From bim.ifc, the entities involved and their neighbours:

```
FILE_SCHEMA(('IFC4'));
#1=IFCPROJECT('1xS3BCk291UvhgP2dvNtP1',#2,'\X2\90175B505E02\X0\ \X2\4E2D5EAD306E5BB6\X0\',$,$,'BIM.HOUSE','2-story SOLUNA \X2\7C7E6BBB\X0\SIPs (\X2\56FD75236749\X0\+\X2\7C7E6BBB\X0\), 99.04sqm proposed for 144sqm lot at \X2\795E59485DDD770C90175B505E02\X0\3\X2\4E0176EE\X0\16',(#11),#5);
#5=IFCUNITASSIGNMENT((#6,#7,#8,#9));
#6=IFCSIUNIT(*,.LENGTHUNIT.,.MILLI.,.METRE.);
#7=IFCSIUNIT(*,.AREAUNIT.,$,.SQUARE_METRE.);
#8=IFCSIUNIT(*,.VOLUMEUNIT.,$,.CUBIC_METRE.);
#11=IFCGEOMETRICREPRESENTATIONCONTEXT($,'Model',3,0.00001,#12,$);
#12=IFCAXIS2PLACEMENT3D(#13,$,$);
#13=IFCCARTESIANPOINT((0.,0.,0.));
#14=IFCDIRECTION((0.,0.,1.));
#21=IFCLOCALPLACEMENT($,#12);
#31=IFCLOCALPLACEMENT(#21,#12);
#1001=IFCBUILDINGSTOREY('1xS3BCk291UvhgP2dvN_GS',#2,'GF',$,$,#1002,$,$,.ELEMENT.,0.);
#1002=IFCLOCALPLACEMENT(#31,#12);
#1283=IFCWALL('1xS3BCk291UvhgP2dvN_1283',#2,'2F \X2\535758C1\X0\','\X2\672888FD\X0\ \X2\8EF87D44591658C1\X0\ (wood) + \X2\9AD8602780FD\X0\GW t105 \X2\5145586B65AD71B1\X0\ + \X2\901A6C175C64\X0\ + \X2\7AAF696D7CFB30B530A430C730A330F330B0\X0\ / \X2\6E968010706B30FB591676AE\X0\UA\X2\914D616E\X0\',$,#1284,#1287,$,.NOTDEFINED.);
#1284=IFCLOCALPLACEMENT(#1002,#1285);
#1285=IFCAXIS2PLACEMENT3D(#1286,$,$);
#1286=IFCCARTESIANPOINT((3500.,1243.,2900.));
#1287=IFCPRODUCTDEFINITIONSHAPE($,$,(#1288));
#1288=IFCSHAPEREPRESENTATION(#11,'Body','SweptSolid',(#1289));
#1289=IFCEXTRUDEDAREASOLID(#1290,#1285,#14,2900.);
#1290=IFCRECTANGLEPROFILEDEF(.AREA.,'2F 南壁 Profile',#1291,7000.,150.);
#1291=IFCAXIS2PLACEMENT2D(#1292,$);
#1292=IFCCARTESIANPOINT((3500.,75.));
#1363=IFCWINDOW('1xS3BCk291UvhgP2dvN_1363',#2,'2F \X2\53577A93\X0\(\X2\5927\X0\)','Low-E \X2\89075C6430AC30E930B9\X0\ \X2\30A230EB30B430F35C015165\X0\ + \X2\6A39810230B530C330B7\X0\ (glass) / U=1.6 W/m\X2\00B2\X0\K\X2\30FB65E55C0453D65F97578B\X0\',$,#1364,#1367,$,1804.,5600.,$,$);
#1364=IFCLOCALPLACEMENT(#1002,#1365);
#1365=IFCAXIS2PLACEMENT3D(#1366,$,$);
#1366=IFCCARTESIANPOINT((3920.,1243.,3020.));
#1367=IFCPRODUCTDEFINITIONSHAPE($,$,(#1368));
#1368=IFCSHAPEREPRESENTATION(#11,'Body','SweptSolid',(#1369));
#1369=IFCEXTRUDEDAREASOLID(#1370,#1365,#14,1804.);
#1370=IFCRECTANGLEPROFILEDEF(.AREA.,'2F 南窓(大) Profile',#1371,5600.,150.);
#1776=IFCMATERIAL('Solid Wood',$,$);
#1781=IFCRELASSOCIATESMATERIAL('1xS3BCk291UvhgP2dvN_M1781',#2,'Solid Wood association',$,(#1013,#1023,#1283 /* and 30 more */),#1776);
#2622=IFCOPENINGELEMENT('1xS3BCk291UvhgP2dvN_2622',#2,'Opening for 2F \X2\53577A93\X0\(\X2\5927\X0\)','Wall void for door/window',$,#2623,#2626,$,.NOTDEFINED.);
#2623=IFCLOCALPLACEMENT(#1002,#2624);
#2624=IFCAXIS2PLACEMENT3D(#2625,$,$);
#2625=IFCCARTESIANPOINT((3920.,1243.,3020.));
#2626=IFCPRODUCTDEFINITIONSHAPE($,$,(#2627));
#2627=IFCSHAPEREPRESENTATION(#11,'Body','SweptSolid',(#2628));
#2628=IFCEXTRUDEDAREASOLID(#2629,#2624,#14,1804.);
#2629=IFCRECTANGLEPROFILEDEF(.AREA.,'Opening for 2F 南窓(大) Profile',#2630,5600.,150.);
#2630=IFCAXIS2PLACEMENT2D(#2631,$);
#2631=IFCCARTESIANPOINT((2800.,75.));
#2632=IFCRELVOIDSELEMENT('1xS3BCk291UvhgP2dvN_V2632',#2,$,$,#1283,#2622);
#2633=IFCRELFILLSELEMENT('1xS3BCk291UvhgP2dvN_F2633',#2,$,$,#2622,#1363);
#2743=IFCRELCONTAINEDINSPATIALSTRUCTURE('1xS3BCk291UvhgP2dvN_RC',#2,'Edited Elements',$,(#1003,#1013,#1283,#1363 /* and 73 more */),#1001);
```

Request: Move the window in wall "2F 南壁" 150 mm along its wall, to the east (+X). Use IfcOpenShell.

```python
import ifcopenshell
import ifcopenshell.api.geometry
import ifcopenshell.util.placement
import ifcopenshell.util.unit

model = ifcopenshell.open("bim.ifc")
unit_scale = ifcopenshell.util.unit.calculate_unit_scale(model)

window = model.by_guid("1xS3BCk291UvhgP2dvN_1363")
opening = window.FillsVoids[0].RelatingOpeningElement
wall = opening.VoidsElements[0].RelatingBuildingElement

wall_matrix = ifcopenshell.util.placement.get_local_placement(wall.ObjectPlacement)
shift = wall_matrix[:3, 0] * 0.15 / unit_scale
before = ifcopenshell.util.placement.get_local_placement(window.ObjectPlacement)[:3, 3].copy()

# The window is not placed relative to its opening, so move both.
for product in (opening, window):
    matrix = ifcopenshell.util.placement.get_local_placement(product.ObjectPlacement)
    matrix[:3, 3] += shift
    ifcopenshell.api.geometry.edit_object_placement(model, product=product, matrix=matrix, is_si=False)

after = ifcopenshell.util.placement.get_local_placement(window.ObjectPlacement)[:3, 3]
print("window moved by", (after - before).round(3) + 0.0)

model.write("bim_edited.ifc")
```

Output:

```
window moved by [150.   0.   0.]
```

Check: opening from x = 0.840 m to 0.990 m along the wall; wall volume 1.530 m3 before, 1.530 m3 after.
